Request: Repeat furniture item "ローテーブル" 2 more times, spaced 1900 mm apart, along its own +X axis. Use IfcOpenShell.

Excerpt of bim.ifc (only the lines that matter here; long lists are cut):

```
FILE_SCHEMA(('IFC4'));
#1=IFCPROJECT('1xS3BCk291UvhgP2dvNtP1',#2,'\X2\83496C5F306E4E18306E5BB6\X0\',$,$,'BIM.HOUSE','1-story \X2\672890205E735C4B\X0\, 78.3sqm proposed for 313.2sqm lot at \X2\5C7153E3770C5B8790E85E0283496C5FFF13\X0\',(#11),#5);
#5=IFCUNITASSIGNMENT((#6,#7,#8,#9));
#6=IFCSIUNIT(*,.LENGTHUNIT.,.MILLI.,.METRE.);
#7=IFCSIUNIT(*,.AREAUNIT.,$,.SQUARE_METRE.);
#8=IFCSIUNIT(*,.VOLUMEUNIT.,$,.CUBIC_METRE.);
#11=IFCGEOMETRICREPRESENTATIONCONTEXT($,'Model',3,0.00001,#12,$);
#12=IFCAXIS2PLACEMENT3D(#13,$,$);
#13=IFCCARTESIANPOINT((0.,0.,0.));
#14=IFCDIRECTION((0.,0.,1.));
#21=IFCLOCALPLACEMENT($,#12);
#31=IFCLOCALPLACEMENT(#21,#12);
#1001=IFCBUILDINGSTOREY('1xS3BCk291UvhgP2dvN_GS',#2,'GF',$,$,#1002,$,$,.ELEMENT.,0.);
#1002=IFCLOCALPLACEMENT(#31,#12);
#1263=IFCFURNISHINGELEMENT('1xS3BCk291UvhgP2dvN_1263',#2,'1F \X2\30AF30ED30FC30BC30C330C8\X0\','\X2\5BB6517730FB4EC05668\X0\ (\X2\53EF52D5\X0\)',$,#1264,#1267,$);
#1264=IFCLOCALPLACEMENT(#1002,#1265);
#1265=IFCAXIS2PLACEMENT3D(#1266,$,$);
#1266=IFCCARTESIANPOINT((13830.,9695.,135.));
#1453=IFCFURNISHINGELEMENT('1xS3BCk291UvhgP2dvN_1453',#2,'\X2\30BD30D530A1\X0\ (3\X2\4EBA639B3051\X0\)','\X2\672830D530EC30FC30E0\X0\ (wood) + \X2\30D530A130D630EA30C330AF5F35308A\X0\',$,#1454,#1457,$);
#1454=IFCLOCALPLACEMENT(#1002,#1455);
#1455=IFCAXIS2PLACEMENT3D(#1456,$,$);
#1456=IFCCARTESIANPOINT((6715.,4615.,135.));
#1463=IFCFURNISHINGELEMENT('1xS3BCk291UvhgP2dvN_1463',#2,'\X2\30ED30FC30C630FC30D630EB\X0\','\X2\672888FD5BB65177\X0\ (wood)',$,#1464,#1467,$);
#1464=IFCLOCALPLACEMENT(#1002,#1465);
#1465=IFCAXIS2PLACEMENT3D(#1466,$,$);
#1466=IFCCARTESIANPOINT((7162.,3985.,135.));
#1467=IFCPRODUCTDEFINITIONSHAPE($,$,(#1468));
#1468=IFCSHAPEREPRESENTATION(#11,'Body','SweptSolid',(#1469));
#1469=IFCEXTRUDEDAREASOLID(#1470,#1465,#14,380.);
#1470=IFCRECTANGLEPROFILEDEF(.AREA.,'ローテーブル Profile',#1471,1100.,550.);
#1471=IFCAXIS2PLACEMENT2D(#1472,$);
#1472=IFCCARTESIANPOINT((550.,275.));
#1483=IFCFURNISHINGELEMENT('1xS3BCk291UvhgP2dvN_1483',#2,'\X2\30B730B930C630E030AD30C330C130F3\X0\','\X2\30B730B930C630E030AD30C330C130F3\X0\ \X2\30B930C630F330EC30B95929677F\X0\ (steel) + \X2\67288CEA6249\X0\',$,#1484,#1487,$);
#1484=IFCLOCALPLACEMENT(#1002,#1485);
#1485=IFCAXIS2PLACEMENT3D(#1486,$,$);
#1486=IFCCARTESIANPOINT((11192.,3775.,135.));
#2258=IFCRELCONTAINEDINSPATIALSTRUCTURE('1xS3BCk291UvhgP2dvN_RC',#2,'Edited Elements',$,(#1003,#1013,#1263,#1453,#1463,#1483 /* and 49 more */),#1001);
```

```python
import ifcopenshell
import ifcopenshell.api.geometry
import ifcopenshell.api.root
import ifcopenshell.util.element
import ifcopenshell.util.placement
import ifcopenshell.util.unit

model = ifcopenshell.open("bim.ifc")
unit_scale = ifcopenshell.util.unit.calculate_unit_scale(model)


def reuse_history(source, copy):
    """copy_class also copies each property set's owner history, people and application; keep the originals."""
    for rel in copy.IsDefinedBy:
        if rel.is_a("IfcRelDefinesByProperties") and (history := rel.RelatingPropertyDefinition.OwnerHistory):
            rel.RelatingPropertyDefinition.OwnerHistory = source.OwnerHistory
            ifcopenshell.util.element.remove_deep2(model, history)


source = model.by_guid("1xS3BCk291UvhgP2dvN_1463")
base = ifcopenshell.util.placement.get_local_placement(source.ObjectPlacement)
step = base[:3, 0] * 1.9 / unit_scale

for i in range(1, 3):
    copy = ifcopenshell.api.root.copy_class(model, product=source)
    copy.Representation = ifcopenshell.util.element.copy_deep(
        model, source.Representation, exclude=["IfcGeometricRepresentationContext", "IfcRepresentationMap"]
    )
    reuse_history(source, copy)
    matrix = base.copy()
    matrix[:3, 3] += i * step
    print("added at", matrix[:3, 3].round(3) + 0.0)
    ifcopenshell.api.geometry.edit_object_placement(model, product=copy, matrix=matrix, is_si=False)

model.write("bim_rev.ifc")
```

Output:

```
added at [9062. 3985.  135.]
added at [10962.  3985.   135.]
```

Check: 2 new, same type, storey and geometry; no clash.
